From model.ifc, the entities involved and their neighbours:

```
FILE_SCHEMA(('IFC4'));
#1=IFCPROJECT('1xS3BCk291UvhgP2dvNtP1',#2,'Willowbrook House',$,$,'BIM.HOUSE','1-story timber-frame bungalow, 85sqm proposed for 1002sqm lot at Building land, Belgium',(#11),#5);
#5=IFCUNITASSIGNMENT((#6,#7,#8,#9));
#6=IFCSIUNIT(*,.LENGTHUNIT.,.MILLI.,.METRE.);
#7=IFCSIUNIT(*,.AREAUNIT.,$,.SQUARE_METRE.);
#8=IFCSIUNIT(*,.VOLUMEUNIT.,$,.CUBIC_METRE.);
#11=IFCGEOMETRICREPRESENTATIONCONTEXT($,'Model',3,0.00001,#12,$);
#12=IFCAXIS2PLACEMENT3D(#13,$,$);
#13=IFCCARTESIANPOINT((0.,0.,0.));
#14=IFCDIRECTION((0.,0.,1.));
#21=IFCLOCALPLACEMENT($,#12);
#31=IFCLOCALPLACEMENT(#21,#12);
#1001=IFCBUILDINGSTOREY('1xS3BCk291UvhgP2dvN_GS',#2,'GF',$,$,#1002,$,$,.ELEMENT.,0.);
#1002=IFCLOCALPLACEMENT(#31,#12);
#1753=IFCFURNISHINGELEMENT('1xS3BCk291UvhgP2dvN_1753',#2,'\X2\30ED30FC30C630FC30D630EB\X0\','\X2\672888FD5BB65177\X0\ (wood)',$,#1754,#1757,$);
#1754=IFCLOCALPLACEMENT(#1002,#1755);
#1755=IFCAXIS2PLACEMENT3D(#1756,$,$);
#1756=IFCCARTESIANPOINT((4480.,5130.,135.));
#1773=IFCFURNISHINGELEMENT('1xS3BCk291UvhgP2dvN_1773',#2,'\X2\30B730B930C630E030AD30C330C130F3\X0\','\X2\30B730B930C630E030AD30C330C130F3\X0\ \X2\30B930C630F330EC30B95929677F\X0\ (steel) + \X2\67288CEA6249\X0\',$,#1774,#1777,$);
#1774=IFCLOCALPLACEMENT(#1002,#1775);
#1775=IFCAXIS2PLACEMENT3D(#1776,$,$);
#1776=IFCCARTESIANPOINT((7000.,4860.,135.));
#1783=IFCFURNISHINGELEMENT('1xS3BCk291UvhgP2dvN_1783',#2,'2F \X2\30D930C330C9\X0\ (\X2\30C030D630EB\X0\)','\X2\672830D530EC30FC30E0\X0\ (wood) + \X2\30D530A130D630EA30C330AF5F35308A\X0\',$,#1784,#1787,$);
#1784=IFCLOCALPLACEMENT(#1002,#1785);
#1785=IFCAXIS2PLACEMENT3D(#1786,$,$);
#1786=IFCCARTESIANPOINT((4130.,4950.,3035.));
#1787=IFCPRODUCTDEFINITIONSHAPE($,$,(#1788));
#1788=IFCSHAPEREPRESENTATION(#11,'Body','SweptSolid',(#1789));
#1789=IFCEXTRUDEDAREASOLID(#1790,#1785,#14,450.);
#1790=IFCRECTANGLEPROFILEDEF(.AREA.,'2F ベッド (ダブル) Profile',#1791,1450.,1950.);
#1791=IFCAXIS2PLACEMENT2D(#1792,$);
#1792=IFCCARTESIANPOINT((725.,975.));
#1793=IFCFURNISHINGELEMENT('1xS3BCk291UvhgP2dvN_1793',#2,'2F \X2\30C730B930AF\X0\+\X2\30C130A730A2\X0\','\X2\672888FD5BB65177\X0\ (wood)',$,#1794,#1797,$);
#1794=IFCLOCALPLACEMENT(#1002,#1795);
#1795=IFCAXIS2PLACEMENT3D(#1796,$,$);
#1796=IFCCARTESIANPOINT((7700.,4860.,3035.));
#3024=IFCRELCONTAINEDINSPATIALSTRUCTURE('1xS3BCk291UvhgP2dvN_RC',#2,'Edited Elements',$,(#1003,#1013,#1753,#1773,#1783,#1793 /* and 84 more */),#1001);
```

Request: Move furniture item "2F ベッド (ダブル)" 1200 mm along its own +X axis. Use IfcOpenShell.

```python
import ifcopenshell
import ifcopenshell.api.geometry
import ifcopenshell.util.placement

model = ifcopenshell.open("model.ifc")

item = model.by_guid("1xS3BCk291UvhgP2dvN_1783")
matrix = ifcopenshell.util.placement.get_local_placement(item.ObjectPlacement)
matrix[:3, 3] += matrix[:3, 0] * 1200.0
ifcopenshell.api.geometry.edit_object_placement(model, product=item, matrix=matrix, is_si=False)

print(ifcopenshell.util.placement.get_local_placement(item.ObjectPlacement).round(3) + 0.0)

model.write("model_v2.ifc")
```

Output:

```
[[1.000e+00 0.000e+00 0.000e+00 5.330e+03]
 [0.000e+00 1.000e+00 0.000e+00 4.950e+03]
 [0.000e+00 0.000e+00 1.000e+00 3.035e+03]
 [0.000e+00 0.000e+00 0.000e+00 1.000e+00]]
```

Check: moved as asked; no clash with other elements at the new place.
